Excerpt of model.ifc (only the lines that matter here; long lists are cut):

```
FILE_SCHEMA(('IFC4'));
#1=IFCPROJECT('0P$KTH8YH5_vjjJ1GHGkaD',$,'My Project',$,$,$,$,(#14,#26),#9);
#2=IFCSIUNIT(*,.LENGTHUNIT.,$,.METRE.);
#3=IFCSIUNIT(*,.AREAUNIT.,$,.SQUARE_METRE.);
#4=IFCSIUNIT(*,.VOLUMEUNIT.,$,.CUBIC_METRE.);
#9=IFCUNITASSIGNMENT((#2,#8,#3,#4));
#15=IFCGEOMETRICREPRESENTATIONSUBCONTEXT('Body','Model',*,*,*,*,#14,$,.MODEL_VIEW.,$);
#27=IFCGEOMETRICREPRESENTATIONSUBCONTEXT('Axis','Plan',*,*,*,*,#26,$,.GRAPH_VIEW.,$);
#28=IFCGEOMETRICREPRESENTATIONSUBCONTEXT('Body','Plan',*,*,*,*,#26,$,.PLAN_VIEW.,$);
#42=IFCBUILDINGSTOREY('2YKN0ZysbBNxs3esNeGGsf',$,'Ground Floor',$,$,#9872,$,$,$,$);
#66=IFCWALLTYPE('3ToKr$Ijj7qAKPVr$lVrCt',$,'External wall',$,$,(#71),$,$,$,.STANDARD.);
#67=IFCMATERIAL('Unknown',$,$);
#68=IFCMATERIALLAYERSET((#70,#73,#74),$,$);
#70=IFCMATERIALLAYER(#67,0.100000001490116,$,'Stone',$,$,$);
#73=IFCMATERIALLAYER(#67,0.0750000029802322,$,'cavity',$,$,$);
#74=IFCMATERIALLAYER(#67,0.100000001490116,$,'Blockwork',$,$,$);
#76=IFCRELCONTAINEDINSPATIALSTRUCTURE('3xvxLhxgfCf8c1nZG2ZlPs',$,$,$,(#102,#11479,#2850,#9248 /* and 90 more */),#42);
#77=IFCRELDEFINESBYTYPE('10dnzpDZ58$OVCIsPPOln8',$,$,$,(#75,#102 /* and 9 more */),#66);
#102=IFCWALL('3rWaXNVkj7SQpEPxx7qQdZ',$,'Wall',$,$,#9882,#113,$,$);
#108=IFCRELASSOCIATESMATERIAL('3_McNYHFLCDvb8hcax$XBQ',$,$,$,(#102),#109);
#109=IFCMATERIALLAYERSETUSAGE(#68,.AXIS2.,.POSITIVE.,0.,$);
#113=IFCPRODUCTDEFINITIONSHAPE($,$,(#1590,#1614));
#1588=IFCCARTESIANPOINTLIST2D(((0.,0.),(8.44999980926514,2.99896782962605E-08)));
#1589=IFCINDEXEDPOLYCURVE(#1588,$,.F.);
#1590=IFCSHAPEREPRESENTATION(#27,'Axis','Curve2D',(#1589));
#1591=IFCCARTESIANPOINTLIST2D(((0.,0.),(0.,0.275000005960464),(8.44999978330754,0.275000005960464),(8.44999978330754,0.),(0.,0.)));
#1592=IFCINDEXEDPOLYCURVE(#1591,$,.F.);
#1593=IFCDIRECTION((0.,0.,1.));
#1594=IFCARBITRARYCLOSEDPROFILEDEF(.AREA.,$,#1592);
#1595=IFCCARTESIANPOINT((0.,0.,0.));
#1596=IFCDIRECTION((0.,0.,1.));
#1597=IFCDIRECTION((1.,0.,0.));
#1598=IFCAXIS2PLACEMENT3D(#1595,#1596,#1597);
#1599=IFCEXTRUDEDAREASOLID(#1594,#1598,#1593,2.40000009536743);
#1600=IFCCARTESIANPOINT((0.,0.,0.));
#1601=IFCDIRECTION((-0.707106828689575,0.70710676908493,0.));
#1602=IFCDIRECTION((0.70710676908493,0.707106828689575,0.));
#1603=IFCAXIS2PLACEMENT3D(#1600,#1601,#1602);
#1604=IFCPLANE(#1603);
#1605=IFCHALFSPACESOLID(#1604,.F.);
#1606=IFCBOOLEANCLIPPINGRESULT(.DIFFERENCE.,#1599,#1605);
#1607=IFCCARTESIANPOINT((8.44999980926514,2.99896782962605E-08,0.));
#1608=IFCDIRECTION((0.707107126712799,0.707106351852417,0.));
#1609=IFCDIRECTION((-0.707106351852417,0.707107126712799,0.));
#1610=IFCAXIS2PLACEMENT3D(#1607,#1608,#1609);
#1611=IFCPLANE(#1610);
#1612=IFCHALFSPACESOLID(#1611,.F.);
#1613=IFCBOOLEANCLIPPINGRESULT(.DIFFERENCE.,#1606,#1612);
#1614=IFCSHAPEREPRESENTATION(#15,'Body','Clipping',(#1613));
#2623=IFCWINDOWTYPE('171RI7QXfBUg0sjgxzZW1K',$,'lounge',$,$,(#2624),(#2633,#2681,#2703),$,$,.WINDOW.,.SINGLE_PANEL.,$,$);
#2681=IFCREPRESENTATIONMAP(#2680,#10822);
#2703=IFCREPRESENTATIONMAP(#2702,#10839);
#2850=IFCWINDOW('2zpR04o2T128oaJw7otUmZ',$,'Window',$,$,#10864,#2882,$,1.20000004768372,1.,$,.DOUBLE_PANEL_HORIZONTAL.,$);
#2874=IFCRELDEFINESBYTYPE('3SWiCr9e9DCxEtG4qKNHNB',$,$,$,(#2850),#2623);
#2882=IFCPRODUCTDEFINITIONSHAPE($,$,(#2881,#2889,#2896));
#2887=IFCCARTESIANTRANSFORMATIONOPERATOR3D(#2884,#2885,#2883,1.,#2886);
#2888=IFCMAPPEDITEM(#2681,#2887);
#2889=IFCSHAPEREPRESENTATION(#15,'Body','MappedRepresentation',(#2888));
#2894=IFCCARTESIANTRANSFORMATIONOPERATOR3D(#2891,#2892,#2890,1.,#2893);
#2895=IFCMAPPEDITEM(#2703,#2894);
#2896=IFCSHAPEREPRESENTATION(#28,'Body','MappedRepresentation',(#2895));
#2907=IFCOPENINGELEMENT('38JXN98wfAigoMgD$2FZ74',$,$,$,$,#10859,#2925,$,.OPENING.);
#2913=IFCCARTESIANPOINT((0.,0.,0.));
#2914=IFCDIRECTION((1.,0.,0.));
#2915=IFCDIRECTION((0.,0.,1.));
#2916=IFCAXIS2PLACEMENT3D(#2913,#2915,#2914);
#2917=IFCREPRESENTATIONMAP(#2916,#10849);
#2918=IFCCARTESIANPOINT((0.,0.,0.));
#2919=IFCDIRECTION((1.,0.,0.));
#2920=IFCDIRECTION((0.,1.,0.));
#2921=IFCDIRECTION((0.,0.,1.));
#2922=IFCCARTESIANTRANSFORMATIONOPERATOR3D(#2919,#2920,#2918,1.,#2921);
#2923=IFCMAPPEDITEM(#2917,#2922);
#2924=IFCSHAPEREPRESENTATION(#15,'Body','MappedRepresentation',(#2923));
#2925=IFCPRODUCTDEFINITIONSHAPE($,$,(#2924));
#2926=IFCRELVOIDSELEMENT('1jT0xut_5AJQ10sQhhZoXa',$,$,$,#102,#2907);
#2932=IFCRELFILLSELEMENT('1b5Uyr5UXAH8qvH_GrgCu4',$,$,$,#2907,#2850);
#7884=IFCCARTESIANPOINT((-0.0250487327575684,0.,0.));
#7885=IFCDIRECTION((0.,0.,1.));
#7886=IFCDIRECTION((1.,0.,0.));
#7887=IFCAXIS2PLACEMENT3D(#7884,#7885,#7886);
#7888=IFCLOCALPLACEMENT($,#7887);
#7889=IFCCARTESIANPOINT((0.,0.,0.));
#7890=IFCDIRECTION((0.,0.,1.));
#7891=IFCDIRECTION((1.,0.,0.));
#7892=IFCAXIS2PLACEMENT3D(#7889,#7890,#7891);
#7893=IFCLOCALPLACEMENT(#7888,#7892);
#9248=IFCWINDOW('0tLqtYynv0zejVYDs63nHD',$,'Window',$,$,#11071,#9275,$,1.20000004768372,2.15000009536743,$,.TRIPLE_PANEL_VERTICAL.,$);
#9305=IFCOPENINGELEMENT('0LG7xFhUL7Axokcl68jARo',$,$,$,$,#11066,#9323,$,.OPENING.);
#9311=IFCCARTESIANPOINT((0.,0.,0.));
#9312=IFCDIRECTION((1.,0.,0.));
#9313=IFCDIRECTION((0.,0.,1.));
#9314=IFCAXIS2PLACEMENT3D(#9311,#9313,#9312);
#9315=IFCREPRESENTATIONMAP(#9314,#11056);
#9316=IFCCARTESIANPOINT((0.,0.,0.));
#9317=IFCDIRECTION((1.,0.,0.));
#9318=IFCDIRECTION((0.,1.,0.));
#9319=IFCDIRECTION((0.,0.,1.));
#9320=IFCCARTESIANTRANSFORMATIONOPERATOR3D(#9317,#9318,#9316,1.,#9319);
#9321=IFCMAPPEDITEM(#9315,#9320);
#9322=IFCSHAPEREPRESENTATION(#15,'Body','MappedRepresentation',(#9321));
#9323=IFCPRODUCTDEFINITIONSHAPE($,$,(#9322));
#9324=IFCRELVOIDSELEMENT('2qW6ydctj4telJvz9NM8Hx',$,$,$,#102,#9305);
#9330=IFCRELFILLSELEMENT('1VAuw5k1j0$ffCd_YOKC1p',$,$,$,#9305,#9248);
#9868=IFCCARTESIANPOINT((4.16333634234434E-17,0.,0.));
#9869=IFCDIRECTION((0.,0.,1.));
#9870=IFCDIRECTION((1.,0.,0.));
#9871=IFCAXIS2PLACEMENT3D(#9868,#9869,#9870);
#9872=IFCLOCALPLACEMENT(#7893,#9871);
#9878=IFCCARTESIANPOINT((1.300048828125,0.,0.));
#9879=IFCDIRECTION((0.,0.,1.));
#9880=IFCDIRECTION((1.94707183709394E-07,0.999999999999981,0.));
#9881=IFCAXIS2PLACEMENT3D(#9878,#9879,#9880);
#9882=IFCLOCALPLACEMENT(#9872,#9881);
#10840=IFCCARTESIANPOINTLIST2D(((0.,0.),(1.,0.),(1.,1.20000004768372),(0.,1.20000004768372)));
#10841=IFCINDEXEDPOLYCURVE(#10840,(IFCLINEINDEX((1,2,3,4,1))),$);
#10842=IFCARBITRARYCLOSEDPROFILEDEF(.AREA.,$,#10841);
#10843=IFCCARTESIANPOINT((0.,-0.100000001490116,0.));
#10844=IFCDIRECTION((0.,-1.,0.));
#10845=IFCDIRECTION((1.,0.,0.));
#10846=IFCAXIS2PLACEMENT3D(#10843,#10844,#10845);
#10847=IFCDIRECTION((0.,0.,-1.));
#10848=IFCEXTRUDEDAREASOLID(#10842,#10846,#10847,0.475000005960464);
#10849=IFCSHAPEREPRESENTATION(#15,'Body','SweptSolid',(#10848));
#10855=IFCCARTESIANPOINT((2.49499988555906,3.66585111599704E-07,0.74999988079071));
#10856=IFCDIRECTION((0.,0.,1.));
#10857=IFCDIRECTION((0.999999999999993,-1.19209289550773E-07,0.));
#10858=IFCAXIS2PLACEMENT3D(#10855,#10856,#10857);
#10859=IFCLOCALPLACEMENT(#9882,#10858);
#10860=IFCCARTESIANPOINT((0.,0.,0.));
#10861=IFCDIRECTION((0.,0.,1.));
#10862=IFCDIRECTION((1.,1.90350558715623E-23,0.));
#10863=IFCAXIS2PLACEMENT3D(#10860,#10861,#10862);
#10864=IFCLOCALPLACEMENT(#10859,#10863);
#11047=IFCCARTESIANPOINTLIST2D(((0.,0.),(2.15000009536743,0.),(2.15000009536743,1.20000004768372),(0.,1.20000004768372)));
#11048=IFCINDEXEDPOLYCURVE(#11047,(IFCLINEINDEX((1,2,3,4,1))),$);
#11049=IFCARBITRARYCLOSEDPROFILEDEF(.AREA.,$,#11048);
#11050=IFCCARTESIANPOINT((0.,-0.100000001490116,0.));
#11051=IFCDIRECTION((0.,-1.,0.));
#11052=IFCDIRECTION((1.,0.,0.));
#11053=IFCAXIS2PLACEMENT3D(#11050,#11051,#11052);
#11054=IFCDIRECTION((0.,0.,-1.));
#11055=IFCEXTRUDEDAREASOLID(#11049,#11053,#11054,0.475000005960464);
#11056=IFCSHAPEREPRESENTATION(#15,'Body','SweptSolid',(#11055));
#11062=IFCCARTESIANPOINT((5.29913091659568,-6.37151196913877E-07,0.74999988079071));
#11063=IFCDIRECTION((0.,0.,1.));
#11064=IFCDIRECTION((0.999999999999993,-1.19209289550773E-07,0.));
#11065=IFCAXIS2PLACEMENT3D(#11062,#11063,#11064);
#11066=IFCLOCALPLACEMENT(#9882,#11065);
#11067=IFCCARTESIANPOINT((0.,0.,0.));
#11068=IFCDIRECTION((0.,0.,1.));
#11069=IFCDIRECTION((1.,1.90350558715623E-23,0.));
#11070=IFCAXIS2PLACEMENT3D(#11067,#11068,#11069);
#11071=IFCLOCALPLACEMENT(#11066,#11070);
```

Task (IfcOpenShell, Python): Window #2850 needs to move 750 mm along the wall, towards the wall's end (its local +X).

```python
import ifcopenshell
import ifcopenshell.api.geometry
import ifcopenshell.util.placement
import ifcopenshell.util.unit

model = ifcopenshell.open("model.ifc")
unit_scale = ifcopenshell.util.unit.calculate_unit_scale(model)

window = model.by_id(2850)
opening = window.FillsVoids[0].RelatingOpeningElement
wall = opening.VoidsElements[0].RelatingBuildingElement

wall_matrix = ifcopenshell.util.placement.get_local_placement(wall.ObjectPlacement)
shift = wall_matrix[:3, 0] * 0.75 / unit_scale
before = ifcopenshell.util.placement.get_local_placement(window.ObjectPlacement)[:3, 3].copy()

# The window is placed relative to its opening, so it follows when the opening moves.
matrix = ifcopenshell.util.placement.get_local_placement(opening.ObjectPlacement)
matrix[:3, 3] += shift
ifcopenshell.api.geometry.edit_object_placement(
    model, product=opening, matrix=matrix, is_si=False, should_transform_children=True
)

after = ifcopenshell.util.placement.get_local_placement(window.ObjectPlacement)[:3, 3]
print("window moved by", (after - before).round(3) + 0.0)

model.write("model-out.ifc")
```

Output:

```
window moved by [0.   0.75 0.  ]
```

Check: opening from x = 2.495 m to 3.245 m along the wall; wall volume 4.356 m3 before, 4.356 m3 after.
